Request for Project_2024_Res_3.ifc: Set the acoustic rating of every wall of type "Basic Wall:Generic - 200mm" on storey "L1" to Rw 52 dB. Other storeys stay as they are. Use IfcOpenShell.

First a look at what the model holds.

```python
import ifcopenshell
import ifcopenshell.util.element

model = ifcopenshell.open("Project_2024_Res_3.ifc")
print(model.schema)
storey = next(s for s in model.by_type("IfcBuildingStorey") if s.Name == "L1")
walls = [e for e in ifcopenshell.util.element.get_decomposition(storey) if e.is_a("IfcWall")]
seen = {}
for e in walls:
    element_type = ifcopenshell.util.element.get_type(e)
    key = (element_type.Name if element_type != e and element_type else None, ifcopenshell.util.element.get_pset(e, "Pset_WallCommon", "AcousticRating"))
    seen[key] = seen.get(key, 0) + 1
for (name, value), count in sorted(seen.items(), key=str):
    print(count, "x", name, "|", value)
```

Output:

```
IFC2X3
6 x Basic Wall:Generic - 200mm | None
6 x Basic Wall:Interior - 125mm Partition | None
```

```python
import ifcopenshell
import ifcopenshell.api.pset
import ifcopenshell.util.element

model = ifcopenshell.open("Project_2024_Res_3.ifc")

storey = next(s for s in model.by_type("IfcBuildingStorey") if s.Name == "L1")
walls = [e for e in ifcopenshell.util.element.get_decomposition(storey) if e.is_a("IfcWall")]

count = 0
for e in walls:
    element_type = ifcopenshell.util.element.get_type(e)
    if element_type in (None, e) or element_type.Name != "Basic Wall:Generic - 200mm":
        continue
    # add_pset returns the element's existing set when there is one.
    pset = ifcopenshell.api.pset.add_pset(model, product=e, name="Pset_WallCommon")
    ifcopenshell.api.pset.edit_pset(model, pset=pset, properties={"AcousticRating": "Rw 52 dB"})
    count += 1

print(count, "walls updated")

model.write("Project_2024_Res_3_v2.ifc")
```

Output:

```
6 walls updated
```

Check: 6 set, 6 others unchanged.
